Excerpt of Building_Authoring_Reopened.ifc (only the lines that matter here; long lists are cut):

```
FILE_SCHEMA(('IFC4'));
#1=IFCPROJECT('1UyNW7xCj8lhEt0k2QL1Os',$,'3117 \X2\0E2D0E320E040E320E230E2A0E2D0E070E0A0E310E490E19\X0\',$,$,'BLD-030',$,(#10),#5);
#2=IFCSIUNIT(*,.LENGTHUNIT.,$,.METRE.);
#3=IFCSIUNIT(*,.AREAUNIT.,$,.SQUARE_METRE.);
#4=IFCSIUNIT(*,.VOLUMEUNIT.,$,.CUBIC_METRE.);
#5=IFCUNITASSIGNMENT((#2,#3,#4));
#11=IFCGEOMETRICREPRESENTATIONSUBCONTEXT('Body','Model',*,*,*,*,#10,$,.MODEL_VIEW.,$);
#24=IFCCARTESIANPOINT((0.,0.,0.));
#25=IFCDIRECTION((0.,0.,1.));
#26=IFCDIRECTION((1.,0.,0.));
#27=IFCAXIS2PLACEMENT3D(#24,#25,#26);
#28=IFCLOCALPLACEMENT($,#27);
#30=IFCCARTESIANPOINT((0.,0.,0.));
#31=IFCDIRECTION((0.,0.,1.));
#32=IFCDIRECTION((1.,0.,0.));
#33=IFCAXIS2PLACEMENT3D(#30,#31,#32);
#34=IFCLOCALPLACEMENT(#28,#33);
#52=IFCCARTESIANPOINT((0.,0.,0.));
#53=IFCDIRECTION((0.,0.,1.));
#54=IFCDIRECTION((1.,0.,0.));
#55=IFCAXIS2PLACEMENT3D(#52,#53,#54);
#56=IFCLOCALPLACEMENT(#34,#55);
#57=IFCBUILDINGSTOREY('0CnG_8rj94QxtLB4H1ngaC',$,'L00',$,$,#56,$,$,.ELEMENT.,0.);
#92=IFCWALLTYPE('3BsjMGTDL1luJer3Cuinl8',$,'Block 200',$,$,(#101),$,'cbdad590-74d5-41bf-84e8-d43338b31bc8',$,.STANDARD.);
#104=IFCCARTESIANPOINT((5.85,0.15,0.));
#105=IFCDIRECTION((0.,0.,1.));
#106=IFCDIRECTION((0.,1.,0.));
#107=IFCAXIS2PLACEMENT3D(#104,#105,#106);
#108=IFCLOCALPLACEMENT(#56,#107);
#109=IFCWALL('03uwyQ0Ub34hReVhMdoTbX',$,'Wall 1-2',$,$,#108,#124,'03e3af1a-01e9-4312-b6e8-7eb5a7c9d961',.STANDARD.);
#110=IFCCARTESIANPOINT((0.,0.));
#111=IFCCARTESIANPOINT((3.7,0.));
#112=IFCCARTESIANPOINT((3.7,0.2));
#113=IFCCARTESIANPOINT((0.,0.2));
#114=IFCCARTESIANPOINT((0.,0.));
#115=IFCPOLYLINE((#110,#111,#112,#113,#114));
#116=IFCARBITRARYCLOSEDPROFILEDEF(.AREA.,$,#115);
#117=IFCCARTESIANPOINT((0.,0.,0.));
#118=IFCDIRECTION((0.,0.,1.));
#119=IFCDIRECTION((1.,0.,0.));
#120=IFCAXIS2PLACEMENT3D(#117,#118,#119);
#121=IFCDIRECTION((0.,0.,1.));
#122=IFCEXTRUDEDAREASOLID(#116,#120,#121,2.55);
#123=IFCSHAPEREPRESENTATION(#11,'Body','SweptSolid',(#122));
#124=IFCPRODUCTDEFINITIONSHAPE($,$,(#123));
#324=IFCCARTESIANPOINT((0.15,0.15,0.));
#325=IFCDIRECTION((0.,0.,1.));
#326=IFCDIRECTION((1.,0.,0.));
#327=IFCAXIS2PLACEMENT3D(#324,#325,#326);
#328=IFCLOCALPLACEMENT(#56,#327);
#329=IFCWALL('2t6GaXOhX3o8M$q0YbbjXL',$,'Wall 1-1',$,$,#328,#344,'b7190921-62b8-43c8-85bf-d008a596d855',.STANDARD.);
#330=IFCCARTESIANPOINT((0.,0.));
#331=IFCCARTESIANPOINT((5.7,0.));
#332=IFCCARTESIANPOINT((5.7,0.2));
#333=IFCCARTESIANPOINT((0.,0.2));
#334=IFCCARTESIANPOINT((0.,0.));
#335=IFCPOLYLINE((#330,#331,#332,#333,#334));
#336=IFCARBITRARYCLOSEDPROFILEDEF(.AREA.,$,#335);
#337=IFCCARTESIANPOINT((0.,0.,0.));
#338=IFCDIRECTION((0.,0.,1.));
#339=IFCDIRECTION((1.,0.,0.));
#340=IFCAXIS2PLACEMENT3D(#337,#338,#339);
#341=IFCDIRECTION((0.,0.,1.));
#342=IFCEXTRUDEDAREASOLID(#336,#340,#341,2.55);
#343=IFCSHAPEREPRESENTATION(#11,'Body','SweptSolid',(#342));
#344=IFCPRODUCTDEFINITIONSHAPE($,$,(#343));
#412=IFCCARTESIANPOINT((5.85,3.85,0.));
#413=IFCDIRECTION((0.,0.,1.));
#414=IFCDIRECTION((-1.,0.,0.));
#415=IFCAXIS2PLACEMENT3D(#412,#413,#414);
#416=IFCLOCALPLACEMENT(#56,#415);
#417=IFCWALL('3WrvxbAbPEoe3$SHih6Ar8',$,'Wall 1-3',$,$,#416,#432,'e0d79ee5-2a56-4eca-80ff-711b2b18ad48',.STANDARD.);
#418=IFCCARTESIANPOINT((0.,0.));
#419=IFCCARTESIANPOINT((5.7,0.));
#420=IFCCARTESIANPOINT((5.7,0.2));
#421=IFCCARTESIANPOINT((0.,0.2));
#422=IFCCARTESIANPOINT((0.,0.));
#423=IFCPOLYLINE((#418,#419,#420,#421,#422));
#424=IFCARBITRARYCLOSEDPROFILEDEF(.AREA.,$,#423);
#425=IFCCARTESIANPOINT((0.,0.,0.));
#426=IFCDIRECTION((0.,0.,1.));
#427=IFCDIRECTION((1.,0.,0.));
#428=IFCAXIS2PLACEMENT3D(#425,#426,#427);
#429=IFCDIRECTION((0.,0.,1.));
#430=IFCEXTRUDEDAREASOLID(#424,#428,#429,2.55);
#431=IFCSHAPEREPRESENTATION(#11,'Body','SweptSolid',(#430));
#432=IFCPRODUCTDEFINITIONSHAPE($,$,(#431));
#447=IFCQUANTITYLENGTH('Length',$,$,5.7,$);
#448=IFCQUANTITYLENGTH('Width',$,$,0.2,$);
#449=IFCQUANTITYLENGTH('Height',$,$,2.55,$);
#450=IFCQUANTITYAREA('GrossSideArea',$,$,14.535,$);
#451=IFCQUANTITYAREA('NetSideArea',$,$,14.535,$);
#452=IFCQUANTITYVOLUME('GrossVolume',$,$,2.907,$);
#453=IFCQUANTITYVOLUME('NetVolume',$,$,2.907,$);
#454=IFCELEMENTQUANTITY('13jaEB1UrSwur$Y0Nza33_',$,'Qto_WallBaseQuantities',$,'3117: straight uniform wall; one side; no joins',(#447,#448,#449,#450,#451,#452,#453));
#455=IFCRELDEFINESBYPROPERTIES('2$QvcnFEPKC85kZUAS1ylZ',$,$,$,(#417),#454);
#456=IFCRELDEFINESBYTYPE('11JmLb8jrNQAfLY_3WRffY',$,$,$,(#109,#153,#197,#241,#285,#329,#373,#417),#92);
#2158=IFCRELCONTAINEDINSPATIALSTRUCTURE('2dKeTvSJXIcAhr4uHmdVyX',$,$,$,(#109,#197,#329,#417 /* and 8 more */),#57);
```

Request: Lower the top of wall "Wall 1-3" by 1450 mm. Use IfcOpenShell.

```python
import ifcopenshell
import ifcopenshell.api.pset
import ifcopenshell.geom
import ifcopenshell.util.element
import ifcopenshell.util.representation
import ifcopenshell.util.shape
import ifcopenshell.util.unit

model = ifcopenshell.open("Building_Authoring_Reopened.ifc")
unit_scale = ifcopenshell.util.unit.calculate_unit_scale(model)
area_scale = ifcopenshell.util.unit.calculate_unit_scale(model, "AREAUNIT")
volume_scale = ifcopenshell.util.unit.calculate_unit_scale(model, "VOLUMEUNIT")
settings = ifcopenshell.geom.settings()


def volume(element):
    """Net volume in cubic metres, openings subtracted."""
    shape = ifcopenshell.geom.create_shape(settings, element)
    return ifcopenshell.util.shape.get_volume(shape.geometry)


wall = model.by_guid("3WrvxbAbPEoe3$SHih6Ar8")
before = volume(wall)

body = ifcopenshell.util.representation.get_representation(wall, "Model", "Body")
solid = body.Items[0]
old_height = solid.Depth
solid.Depth -= 1.45 / unit_scale
after = volume(wall)
thickness = 0.2  # wall thickness in metres

# Update the stored height, areas and volumes.
qto = model.by_id(ifcopenshell.util.element.get_pset(wall, "Qto_WallBaseQuantities", should_inherit=False)["id"])
ifcopenshell.api.pset.edit_qto(model, qto=qto, properties={
    "Height": solid.Depth,
    "GrossSideArea": ifcopenshell.util.element.get_pset(wall, "Qto_WallBaseQuantities", "GrossSideArea") * solid.Depth / old_height,
    "NetSideArea": after / thickness / area_scale,
    "GrossVolume": ifcopenshell.util.element.get_pset(wall, "Qto_WallBaseQuantities", "GrossVolume") * solid.Depth / old_height,
    "NetVolume": after / volume_scale,
})

print(f"height {old_height:g} -> {solid.Depth:g}, volume {before:.3f} -> {after:.3f} m3")

model.write("Building_Authoring_Reopened_rev.ifc")
```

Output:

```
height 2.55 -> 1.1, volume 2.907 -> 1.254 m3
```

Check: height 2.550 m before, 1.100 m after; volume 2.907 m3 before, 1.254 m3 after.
